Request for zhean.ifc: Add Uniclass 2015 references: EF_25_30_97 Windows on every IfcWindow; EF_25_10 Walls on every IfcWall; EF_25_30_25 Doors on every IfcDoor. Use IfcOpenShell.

First a look at what the model holds.

```python
import ifcopenshell

model = ifcopenshell.open("zhean.ifc")
print(model.schema)
print("classifications:", [c.Name for c in model.by_type("IfcClassification")])
for ifc_class in ("IfcDoor", "IfcRoof", "IfcStair", "IfcWall", "IfcWindow"):
    print(ifc_class, len(model.by_type(ifc_class)))
```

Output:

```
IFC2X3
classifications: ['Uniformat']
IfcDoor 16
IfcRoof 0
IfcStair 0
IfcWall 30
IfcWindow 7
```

```python
import ifcopenshell
import ifcopenshell.api.classification

model = ifcopenshell.open("zhean.ifc")

# IFC2X3 requires Source and Edition and has no link from the project to the system.
system = model.create_entity("IfcClassification", Source="NBS", Edition="2015", Name="Uniclass 2015")

codes = {
    "IfcWindow": ("EF_25_30_97", "Windows"),
    "IfcWall": ("EF_25_10", "Walls"),
    "IfcDoor": ("EF_25_30_25", "Doors"),
}
for ifc_class, (code, name) in codes.items():
    products = model.by_type(ifc_class)
    ifcopenshell.api.classification.add_reference(
        model, products=products, classification=system, identification=code, name=name
    )
    print(code, len(products))

model.write("zhean_v2.ifc")
```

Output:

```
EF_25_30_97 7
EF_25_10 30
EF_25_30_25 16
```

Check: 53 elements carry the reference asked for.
